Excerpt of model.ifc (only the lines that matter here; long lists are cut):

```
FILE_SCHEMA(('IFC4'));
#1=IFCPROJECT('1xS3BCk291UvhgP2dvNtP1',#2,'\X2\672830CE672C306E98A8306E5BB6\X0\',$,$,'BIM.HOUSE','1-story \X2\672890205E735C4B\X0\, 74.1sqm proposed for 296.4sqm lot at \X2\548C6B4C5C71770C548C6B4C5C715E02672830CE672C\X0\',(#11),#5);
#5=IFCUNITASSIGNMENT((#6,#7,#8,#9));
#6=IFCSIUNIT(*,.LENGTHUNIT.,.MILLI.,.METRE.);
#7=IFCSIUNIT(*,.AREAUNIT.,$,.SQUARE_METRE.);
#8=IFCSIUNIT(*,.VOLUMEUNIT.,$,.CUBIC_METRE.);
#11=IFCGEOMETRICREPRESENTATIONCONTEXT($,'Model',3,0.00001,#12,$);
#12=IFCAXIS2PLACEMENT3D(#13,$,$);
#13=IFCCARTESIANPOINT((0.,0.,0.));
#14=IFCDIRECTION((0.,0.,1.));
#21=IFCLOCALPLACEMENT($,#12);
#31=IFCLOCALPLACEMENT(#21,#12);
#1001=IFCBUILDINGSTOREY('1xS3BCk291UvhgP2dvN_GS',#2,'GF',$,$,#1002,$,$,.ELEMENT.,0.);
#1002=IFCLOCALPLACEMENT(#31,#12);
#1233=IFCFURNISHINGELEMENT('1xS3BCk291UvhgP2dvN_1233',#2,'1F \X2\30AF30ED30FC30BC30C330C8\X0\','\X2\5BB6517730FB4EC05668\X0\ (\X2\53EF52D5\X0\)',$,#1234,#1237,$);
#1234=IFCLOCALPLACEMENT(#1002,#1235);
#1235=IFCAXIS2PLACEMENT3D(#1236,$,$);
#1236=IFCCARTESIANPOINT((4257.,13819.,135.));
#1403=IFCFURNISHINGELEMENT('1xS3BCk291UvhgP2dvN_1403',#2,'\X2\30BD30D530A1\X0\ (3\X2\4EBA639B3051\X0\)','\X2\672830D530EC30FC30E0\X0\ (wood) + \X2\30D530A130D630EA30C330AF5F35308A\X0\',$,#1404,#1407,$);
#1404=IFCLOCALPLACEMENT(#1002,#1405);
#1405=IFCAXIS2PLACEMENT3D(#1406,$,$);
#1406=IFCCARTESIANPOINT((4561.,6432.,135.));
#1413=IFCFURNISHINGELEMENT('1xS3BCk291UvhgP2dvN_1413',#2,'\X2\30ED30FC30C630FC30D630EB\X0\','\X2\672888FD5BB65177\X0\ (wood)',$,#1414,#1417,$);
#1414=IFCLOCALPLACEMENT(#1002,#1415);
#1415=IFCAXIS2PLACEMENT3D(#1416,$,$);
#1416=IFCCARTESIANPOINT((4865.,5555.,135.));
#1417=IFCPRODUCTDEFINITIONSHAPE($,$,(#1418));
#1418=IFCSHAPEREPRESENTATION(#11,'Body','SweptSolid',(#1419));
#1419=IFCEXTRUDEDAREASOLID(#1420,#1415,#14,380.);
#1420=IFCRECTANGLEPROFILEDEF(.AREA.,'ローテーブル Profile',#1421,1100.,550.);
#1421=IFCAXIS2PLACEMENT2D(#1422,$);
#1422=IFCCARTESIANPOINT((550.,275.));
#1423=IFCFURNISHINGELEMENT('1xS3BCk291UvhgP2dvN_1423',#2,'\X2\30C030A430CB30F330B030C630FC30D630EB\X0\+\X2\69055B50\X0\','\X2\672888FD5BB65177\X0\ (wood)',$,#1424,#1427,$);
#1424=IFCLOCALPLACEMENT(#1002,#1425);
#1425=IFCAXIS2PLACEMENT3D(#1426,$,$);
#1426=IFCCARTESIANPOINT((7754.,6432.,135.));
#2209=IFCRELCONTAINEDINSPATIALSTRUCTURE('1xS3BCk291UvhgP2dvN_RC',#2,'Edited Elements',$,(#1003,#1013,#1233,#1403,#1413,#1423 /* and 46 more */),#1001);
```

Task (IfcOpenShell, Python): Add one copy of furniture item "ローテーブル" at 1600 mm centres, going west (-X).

```python
import numpy as np
import ifcopenshell
import ifcopenshell.api.geometry
import ifcopenshell.api.root
import ifcopenshell.util.element
import ifcopenshell.util.placement
import ifcopenshell.util.unit

model = ifcopenshell.open("model.ifc")
unit_scale = ifcopenshell.util.unit.calculate_unit_scale(model)


def reuse_history(source, copy):
    """copy_class also copies each property set's owner history, people and application; keep the originals."""
    for rel in copy.IsDefinedBy:
        if rel.is_a("IfcRelDefinesByProperties") and (history := rel.RelatingPropertyDefinition.OwnerHistory):
            rel.RelatingPropertyDefinition.OwnerHistory = source.OwnerHistory
            ifcopenshell.util.element.remove_deep2(model, history)


source = model.by_guid("1xS3BCk291UvhgP2dvN_1413")
base = ifcopenshell.util.placement.get_local_placement(source.ObjectPlacement)
step = np.array([-1.0, 0.0, 0.0]) * 1.6 / unit_scale

for i in range(1, 2):
    copy = ifcopenshell.api.root.copy_class(model, product=source)
    copy.Representation = ifcopenshell.util.element.copy_deep(
        model, source.Representation, exclude=["IfcGeometricRepresentationContext", "IfcRepresentationMap"]
    )
    reuse_history(source, copy)
    matrix = base.copy()
    matrix[:3, 3] += i * step
    print("added at", matrix[:3, 3].round(3) + 0.0)
    ifcopenshell.api.geometry.edit_object_placement(model, product=copy, matrix=matrix, is_si=False)

model.write("model-out.ifc")
```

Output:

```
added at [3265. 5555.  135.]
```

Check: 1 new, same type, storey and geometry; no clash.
